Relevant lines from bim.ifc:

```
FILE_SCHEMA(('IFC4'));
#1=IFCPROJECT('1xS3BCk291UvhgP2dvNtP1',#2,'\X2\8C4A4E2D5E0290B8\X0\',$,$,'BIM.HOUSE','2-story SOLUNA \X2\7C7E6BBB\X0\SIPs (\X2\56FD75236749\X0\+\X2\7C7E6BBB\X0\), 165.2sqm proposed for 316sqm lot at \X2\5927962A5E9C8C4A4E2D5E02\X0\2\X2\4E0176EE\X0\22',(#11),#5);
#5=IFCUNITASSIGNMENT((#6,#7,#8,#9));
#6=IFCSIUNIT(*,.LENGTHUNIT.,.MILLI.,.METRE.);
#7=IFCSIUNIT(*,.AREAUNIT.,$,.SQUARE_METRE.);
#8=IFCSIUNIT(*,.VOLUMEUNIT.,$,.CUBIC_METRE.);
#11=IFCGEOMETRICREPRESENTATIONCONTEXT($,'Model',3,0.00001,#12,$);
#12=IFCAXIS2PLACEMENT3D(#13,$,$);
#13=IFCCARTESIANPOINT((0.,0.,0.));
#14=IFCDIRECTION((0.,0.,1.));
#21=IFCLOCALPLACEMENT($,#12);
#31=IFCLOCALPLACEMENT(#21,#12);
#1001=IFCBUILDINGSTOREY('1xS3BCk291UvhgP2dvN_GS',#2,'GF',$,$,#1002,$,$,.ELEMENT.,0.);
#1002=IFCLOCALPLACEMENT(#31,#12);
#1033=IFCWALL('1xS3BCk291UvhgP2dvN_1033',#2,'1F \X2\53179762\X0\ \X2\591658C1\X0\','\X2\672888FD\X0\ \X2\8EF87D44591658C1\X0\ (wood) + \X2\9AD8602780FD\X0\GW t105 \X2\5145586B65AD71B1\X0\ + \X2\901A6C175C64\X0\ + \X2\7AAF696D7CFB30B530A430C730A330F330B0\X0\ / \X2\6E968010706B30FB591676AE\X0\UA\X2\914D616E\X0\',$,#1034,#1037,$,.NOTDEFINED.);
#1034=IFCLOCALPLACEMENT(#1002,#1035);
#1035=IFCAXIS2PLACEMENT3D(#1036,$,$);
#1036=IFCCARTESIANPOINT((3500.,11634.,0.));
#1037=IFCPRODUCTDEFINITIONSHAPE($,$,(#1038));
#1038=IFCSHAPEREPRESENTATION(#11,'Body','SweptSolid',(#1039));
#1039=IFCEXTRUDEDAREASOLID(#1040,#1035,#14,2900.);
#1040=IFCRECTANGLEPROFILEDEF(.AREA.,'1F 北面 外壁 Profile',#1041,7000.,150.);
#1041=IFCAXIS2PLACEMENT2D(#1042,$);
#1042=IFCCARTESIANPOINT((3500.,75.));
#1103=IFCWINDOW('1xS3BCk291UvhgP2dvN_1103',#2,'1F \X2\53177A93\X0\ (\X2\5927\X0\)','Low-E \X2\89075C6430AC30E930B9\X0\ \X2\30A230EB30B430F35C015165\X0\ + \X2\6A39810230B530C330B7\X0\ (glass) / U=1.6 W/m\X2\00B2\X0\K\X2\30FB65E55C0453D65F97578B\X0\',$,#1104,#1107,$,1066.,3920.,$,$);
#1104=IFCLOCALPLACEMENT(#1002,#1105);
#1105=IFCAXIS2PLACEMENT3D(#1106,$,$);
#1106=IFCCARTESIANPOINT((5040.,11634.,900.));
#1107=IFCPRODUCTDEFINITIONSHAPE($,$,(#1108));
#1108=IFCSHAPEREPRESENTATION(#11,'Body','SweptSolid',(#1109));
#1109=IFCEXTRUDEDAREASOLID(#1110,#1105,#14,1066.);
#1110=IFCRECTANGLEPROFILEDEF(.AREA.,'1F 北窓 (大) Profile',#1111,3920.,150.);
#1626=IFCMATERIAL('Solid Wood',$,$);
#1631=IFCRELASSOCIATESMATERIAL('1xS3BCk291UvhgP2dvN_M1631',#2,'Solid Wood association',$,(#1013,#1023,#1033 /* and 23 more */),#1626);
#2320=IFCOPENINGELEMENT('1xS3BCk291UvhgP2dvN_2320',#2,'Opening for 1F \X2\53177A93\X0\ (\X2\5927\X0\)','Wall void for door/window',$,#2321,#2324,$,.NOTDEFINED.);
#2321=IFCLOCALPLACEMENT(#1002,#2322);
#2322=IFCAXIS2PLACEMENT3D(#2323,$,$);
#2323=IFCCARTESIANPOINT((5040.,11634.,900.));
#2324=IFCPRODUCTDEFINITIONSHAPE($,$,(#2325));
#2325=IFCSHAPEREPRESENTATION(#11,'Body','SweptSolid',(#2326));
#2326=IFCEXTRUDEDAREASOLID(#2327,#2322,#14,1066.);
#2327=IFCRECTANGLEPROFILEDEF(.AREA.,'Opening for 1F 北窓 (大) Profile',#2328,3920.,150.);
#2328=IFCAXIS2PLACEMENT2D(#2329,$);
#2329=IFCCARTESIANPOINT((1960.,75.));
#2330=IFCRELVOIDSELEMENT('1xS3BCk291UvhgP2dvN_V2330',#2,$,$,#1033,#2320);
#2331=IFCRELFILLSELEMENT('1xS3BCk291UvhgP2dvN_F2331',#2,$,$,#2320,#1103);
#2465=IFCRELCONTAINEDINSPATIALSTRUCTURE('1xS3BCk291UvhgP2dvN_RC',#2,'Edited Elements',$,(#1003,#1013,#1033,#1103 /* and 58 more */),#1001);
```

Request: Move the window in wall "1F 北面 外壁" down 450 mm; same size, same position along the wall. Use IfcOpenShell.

```python
import numpy as np
import ifcopenshell
import ifcopenshell.api.geometry
import ifcopenshell.util.placement
import ifcopenshell.util.unit

model = ifcopenshell.open("bim.ifc")
unit_scale = ifcopenshell.util.unit.calculate_unit_scale(model)

window = model.by_id(1103)
opening = window.FillsVoids[0].RelatingOpeningElement
dz = -0.45 / unit_scale

shift = np.array([0.0, 0.0, dz])
# The window is not placed relative to its opening, so move both.
for product in (opening, window):
    matrix = ifcopenshell.util.placement.get_local_placement(product.ObjectPlacement)
    matrix[:3, 3] += shift
    ifcopenshell.api.geometry.edit_object_placement(model, product=product, matrix=matrix, is_si=False)

print(f"moved by {dz * unit_scale:+.3f} m")

model.write("bim_updated.ifc")
```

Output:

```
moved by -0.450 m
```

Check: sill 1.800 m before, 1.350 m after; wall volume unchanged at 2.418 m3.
